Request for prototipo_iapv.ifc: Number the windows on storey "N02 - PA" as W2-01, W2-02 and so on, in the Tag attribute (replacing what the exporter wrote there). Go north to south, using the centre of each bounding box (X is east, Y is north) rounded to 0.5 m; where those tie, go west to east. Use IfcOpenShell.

First a look at what the model holds.

```python
import ifcopenshell
import ifcopenshell.util.element
import ifcopenshell.util.placement

model = ifcopenshell.open("prototipo_iapv.ifc")
print(model.schema)
storey = next(s for s in model.by_type("IfcBuildingStorey") if s.Name == "N02 - PA")
windows = [e for e in ifcopenshell.util.element.get_decomposition(storey) if e.is_a("IfcWindow")]
for e in sorted(windows, key=lambda e: e.id()):
    origin = ifcopenshell.util.placement.get_local_placement(e.ObjectPlacement)[:3, 3]
    print(e.id(), e.Tag, e.Name, origin.round(2) + 0.0, sep=" | ")
```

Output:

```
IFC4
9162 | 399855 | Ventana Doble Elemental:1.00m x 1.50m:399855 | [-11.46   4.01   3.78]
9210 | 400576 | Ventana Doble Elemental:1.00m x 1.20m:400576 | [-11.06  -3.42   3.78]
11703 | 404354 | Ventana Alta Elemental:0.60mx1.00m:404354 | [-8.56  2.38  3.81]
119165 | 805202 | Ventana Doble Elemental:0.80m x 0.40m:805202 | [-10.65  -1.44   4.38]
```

```python
import ifcopenshell
import ifcopenshell.geom
import ifcopenshell.util.element
import ifcopenshell.util.shape

model = ifcopenshell.open("prototipo_iapv.ifc")
settings = ifcopenshell.geom.settings()
settings.set("use-world-coords", True)


def centre(element):
    shape = ifcopenshell.geom.create_shape(settings, element)
    return ifcopenshell.util.shape.get_bbox_centroid(shape.geometry)


storey = next(s for s in model.by_type("IfcBuildingStorey") if s.Name == "N02 - PA")
windows = [e for e in ifcopenshell.util.element.get_decomposition(storey) if e.is_a("IfcWindow")]

# Insertion points can sit at a corner or the storey origin, so sort by the geometry (in metres).
centres = {e: centre(e) for e in windows}
windows.sort(key=lambda e: (-round(centres[e][1] / 0.5), centres[e][0]))

for i, e in enumerate(windows, start=1):
    number = f"W2-{i:02d}"
    e.Tag = number
    print(e.id(), number)

model.write("prototipo_iapv_v2.ifc")
```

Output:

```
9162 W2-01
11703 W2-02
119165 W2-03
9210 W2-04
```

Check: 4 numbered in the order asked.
